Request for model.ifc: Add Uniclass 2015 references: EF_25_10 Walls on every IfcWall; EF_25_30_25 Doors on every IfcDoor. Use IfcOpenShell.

First a look at what the model holds.

```python
import ifcopenshell

model = ifcopenshell.open("model.ifc")
print(model.schema)
print("classifications:", [c.Name for c in model.by_type("IfcClassification")])
for ifc_class in ("IfcDoor", "IfcRoof", "IfcStair", "IfcWall", "IfcWindow"):
    print(ifc_class, len(model.by_type(ifc_class)))
```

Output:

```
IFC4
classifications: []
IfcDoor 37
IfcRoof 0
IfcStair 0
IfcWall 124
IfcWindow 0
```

```python
import ifcopenshell
import ifcopenshell.api.classification

model = ifcopenshell.open("model.ifc")

system = ifcopenshell.api.classification.add_classification(model, classification="Uniclass 2015")

codes = {
    "IfcWall": ("EF_25_10", "Walls"),
    "IfcDoor": ("EF_25_30_25", "Doors"),
}
for ifc_class, (code, name) in codes.items():
    products = model.by_type(ifc_class)
    ifcopenshell.api.classification.add_reference(
        model, products=products, classification=system, identification=code, name=name
    )
    print(code, len(products))

model.write("model-out.ifc")
```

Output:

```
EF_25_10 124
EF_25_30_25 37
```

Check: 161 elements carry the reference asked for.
